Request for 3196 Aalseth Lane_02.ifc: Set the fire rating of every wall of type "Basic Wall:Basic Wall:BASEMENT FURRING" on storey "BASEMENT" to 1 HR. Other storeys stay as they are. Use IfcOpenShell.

First a look at what the model holds.

```python
import ifcopenshell
import ifcopenshell.util.element

model = ifcopenshell.open("3196 Aalseth Lane_02.ifc")
print(model.schema)
storey = next(s for s in model.by_type("IfcBuildingStorey") if s.Name == "BASEMENT")
walls = [e for e in ifcopenshell.util.element.get_decomposition(storey) if e.is_a("IfcWall")]
seen = {}
for e in walls:
    element_type = ifcopenshell.util.element.get_type(e)
    key = (element_type.Name if element_type != e and element_type else None, ifcopenshell.util.element.get_pset(e, "Pset_WallCommon", "FireRating"))
    seen[key] = seen.get(key, 0) + 1
for (name, value), count in sorted(seen.items(), key=str):
    print(count, "x", name, "|", value)
```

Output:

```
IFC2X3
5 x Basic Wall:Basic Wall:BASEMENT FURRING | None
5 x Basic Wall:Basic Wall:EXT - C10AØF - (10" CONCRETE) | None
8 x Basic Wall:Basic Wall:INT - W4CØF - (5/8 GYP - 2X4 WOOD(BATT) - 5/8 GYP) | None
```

```python
import ifcopenshell
import ifcopenshell.api.pset
import ifcopenshell.util.element

model = ifcopenshell.open("3196 Aalseth Lane_02.ifc")

storey = next(s for s in model.by_type("IfcBuildingStorey") if s.Name == "BASEMENT")
walls = [e for e in ifcopenshell.util.element.get_decomposition(storey) if e.is_a("IfcWall")]

count = 0
for e in walls:
    element_type = ifcopenshell.util.element.get_type(e)
    if element_type in (None, e) or element_type.Name != "Basic Wall:Basic Wall:BASEMENT FURRING":
        continue
    # add_pset returns the element's existing set when there is one.
    pset = ifcopenshell.api.pset.add_pset(model, product=e, name="Pset_WallCommon")
    ifcopenshell.api.pset.edit_pset(model, pset=pset, properties={"FireRating": "1 HR"})
    count += 1

print(count, "walls updated")

model.write("3196 Aalseth Lane_02_v2.ifc")
```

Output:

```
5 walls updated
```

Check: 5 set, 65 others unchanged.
